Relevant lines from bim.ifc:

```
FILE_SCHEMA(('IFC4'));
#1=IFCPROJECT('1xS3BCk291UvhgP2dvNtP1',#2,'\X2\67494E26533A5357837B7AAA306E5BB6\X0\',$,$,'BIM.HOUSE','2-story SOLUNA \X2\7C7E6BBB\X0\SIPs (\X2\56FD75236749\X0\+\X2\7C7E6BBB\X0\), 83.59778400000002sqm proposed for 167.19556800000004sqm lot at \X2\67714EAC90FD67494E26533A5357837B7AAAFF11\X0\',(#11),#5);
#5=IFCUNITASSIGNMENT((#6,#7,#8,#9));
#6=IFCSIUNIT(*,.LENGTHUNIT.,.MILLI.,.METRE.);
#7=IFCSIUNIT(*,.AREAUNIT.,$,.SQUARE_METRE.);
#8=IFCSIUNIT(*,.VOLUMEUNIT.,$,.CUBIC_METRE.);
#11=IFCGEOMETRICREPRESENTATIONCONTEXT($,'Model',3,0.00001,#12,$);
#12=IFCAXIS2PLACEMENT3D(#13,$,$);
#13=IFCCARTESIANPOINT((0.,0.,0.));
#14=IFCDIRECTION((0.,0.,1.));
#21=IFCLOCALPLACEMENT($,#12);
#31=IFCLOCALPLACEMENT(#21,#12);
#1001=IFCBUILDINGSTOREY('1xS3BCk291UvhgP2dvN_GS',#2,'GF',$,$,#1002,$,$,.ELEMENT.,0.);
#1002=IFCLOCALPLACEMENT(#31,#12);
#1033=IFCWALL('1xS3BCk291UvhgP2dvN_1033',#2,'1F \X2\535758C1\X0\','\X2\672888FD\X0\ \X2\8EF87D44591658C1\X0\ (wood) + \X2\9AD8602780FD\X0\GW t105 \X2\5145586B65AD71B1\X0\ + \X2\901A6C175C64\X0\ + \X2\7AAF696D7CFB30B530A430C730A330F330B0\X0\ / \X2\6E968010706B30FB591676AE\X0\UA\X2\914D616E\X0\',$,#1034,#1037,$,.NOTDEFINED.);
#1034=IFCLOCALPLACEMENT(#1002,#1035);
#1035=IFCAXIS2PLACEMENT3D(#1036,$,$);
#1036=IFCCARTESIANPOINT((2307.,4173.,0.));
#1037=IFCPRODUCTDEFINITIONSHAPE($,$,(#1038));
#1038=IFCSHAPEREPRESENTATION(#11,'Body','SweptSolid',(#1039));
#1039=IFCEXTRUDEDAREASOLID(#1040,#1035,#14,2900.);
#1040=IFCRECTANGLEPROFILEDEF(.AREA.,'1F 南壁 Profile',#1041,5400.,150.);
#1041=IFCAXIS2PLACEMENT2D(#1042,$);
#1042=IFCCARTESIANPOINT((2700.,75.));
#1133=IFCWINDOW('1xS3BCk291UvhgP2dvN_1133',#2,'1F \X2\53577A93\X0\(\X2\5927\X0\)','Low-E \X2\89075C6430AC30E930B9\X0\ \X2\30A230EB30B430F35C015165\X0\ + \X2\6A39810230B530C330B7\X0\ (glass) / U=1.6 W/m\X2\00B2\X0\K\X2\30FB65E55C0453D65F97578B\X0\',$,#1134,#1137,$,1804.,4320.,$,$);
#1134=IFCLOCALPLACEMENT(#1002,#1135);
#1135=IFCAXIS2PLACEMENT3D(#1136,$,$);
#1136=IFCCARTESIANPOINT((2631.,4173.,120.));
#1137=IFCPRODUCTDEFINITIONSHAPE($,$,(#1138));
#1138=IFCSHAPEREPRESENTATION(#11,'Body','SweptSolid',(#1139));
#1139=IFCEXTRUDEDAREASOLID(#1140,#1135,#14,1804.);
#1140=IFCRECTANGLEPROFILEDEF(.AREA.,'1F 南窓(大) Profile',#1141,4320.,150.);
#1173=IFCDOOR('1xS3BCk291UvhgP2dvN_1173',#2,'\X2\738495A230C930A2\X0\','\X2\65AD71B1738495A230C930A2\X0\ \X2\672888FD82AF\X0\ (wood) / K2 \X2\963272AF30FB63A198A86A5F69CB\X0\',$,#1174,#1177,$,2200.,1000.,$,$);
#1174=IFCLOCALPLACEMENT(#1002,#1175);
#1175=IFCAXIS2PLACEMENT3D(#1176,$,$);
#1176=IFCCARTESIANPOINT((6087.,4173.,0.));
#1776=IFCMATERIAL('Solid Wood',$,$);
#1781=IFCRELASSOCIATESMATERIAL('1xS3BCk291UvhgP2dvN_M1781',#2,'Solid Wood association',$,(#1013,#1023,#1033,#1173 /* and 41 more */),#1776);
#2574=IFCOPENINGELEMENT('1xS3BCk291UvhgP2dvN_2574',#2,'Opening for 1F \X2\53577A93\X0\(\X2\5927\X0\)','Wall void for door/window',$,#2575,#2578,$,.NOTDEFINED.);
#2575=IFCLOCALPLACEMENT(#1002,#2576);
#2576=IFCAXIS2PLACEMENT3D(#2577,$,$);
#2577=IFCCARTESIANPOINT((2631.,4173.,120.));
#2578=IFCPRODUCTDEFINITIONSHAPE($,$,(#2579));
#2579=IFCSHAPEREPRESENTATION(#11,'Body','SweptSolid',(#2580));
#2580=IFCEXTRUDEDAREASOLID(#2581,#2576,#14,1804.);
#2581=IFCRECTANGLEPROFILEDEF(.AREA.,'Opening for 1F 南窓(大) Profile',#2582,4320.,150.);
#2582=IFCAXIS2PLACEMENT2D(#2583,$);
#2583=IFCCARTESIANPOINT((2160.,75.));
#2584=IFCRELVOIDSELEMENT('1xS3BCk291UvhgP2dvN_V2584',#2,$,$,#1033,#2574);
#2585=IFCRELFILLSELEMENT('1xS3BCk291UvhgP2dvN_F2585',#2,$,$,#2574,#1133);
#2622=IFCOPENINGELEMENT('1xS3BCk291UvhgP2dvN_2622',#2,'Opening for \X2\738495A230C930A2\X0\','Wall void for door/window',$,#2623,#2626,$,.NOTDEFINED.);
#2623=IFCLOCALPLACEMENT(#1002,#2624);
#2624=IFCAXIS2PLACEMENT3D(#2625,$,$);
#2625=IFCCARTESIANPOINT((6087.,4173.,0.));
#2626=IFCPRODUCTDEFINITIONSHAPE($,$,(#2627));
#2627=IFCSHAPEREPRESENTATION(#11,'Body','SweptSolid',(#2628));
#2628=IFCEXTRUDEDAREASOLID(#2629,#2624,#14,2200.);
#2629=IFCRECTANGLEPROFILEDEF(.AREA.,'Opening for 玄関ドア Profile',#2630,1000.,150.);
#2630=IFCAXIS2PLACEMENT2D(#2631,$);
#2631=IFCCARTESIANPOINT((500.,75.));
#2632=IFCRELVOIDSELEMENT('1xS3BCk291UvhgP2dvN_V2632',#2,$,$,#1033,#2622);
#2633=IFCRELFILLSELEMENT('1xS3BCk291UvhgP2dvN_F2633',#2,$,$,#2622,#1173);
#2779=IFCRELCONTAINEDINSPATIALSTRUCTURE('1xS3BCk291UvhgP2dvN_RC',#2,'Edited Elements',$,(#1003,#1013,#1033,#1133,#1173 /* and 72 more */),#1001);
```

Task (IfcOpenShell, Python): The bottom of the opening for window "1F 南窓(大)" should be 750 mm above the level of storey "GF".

```python
import numpy as np
import ifcopenshell
import ifcopenshell.api.geometry
import ifcopenshell.geom
import ifcopenshell.util.element
import ifcopenshell.util.placement
import ifcopenshell.util.shape
import ifcopenshell.util.unit

model = ifcopenshell.open("bim.ifc")
unit_scale = ifcopenshell.util.unit.calculate_unit_scale(model)

window = model.by_id(1133)
opening = window.FillsVoids[0].RelatingOpeningElement
storey = ifcopenshell.util.element.get_container(window, ifc_class="IfcBuildingStorey")
level = ifcopenshell.util.placement.get_local_placement(storey.ObjectPlacement)[2, 3]

# The opening's origin need not be at the sill, so measure its lowest point.
shape = ifcopenshell.geom.create_shape(ifcopenshell.geom.settings(), opening)
bottom = ifcopenshell.util.shape.get_shape_bottom_elevation(shape, shape.geometry) / unit_scale
dz = level + 0.75 / unit_scale - bottom

shift = np.array([0.0, 0.0, dz])
# The window is not placed relative to its opening, so move both.
for product in (opening, window):
    matrix = ifcopenshell.util.placement.get_local_placement(product.ObjectPlacement)
    matrix[:3, 3] += shift
    ifcopenshell.api.geometry.edit_object_placement(model, product=product, matrix=matrix, is_si=False)

print(f"moved by {dz * unit_scale:+.3f} m")

model.write("bim_rev.ifc")
```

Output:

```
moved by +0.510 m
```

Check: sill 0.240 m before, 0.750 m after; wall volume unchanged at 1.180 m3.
